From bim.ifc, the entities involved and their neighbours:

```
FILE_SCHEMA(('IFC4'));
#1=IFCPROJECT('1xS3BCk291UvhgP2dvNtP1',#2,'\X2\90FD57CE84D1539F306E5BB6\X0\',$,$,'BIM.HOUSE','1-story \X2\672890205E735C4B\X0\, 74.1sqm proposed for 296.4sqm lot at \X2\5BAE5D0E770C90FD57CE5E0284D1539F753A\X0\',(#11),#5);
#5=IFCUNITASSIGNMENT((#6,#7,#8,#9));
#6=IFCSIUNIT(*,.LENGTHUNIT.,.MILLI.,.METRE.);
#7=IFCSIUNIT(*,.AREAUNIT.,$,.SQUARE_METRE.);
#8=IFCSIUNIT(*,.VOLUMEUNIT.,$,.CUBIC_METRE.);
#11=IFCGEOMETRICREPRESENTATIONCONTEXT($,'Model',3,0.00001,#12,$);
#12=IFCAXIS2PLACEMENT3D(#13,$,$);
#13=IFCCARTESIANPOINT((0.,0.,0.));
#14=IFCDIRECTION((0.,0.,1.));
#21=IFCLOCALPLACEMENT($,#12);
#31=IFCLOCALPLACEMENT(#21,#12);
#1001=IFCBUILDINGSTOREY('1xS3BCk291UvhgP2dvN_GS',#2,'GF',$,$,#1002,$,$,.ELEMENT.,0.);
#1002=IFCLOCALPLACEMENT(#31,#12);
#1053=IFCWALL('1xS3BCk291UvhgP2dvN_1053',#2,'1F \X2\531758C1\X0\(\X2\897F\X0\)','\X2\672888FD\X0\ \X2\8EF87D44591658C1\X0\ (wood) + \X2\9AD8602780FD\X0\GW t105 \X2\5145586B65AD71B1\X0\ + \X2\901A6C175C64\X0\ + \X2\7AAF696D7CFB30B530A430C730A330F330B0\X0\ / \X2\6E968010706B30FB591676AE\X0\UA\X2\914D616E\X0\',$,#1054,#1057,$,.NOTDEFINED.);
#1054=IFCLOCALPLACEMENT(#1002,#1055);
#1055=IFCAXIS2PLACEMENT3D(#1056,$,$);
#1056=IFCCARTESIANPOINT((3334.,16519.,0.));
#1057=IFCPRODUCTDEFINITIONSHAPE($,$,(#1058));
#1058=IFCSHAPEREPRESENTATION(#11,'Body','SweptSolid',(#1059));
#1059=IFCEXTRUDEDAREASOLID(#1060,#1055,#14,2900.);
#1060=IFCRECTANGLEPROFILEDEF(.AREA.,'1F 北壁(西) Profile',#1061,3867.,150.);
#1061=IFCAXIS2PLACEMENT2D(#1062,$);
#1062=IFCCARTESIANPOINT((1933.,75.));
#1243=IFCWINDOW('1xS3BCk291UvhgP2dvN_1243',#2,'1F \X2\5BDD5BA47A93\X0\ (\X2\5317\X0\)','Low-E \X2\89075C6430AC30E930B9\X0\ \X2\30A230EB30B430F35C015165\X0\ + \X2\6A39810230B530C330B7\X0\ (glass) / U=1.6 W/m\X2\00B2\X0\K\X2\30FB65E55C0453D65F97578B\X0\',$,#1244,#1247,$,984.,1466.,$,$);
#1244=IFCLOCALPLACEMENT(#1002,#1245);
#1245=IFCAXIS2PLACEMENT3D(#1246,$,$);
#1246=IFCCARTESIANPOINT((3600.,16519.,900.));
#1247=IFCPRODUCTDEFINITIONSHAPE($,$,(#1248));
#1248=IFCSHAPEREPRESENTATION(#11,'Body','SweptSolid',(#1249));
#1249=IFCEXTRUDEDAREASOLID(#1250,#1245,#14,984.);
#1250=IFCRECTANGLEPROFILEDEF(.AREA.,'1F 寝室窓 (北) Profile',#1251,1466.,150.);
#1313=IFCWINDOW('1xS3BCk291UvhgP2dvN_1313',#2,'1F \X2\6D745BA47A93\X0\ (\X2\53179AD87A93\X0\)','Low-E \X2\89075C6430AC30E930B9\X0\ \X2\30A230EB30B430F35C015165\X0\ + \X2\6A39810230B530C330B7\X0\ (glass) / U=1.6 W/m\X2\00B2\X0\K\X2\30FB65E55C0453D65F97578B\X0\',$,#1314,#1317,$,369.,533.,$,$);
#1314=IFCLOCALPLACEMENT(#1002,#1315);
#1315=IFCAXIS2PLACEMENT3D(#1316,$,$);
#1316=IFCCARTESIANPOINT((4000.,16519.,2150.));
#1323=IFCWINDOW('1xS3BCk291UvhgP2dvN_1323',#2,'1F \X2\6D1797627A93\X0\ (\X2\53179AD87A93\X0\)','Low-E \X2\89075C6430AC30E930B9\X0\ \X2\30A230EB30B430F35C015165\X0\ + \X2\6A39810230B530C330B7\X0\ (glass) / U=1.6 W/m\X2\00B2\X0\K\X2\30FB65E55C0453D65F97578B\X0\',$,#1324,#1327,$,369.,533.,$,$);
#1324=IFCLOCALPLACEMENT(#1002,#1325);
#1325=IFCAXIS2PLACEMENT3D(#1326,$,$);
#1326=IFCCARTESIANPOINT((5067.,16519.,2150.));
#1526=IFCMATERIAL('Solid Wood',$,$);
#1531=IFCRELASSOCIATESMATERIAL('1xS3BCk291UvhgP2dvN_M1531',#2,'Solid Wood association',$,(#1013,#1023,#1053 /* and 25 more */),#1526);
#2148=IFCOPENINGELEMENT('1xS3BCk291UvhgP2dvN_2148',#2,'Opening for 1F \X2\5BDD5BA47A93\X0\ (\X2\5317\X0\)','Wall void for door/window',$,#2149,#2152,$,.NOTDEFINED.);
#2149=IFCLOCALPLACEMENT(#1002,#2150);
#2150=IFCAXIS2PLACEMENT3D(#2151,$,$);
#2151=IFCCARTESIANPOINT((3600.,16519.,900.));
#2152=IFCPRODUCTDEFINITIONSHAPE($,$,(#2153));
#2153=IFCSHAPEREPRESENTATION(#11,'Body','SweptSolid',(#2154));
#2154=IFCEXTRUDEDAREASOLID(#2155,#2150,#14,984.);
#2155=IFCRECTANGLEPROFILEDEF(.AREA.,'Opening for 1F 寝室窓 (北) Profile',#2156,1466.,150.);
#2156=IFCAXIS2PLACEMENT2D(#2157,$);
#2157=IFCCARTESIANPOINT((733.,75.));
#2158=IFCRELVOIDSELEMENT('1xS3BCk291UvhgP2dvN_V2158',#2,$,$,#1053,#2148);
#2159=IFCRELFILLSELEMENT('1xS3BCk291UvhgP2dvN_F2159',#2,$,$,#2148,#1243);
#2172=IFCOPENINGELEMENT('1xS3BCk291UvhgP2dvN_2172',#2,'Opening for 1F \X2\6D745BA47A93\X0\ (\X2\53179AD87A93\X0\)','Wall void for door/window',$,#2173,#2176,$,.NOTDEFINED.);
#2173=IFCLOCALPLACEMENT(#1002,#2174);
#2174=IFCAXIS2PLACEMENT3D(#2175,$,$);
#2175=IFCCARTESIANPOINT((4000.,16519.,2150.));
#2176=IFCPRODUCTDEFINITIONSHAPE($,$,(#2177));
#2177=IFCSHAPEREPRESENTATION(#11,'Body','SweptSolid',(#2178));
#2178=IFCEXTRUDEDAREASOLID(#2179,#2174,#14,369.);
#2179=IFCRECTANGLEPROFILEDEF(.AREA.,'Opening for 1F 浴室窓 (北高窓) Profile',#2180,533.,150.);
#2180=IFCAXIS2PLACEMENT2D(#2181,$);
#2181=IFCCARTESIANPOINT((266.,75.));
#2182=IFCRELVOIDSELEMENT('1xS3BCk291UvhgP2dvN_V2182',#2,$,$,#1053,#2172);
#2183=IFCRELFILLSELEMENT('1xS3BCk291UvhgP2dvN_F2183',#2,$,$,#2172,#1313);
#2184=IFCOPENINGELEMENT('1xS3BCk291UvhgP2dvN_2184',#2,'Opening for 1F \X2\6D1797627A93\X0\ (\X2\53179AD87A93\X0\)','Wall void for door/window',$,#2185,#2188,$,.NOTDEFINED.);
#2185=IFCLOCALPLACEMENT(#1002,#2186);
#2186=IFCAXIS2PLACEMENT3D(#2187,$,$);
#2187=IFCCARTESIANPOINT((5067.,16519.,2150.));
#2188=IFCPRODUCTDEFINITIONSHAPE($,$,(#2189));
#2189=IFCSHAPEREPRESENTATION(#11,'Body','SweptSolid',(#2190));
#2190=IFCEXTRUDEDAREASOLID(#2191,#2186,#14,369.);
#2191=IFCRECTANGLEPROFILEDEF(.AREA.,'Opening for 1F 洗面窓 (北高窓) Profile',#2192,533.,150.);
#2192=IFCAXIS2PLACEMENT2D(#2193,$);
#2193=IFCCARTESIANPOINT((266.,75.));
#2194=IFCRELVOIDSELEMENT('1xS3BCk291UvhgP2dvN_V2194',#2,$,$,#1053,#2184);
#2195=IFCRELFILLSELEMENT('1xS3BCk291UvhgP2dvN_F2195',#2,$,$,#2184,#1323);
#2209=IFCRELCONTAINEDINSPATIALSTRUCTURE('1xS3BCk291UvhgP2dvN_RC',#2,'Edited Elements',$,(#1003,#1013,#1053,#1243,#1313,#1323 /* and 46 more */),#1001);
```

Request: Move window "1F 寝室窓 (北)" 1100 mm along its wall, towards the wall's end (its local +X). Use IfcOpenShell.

```python
import ifcopenshell
import ifcopenshell.api.geometry
import ifcopenshell.util.placement
import ifcopenshell.util.unit

model = ifcopenshell.open("bim.ifc")
unit_scale = ifcopenshell.util.unit.calculate_unit_scale(model)

window = model.by_guid("1xS3BCk291UvhgP2dvN_1243")
opening = window.FillsVoids[0].RelatingOpeningElement
wall = opening.VoidsElements[0].RelatingBuildingElement

wall_matrix = ifcopenshell.util.placement.get_local_placement(wall.ObjectPlacement)
shift = wall_matrix[:3, 0] * 1.1 / unit_scale
before = ifcopenshell.util.placement.get_local_placement(window.ObjectPlacement)[:3, 3].copy()

# The window is not placed relative to its opening, so move both.
for product in (opening, window):
    matrix = ifcopenshell.util.placement.get_local_placement(product.ObjectPlacement)
    matrix[:3, 3] += shift
    ifcopenshell.api.geometry.edit_object_placement(model, product=product, matrix=matrix, is_si=False)

after = ifcopenshell.util.placement.get_local_placement(window.ObjectPlacement)[:3, 3]
print("window moved by", (after - before).round(3) + 0.0)

model.write("bim_v2.ifc")
```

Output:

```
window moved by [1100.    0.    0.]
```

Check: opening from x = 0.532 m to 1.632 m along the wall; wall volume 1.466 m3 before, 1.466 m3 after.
